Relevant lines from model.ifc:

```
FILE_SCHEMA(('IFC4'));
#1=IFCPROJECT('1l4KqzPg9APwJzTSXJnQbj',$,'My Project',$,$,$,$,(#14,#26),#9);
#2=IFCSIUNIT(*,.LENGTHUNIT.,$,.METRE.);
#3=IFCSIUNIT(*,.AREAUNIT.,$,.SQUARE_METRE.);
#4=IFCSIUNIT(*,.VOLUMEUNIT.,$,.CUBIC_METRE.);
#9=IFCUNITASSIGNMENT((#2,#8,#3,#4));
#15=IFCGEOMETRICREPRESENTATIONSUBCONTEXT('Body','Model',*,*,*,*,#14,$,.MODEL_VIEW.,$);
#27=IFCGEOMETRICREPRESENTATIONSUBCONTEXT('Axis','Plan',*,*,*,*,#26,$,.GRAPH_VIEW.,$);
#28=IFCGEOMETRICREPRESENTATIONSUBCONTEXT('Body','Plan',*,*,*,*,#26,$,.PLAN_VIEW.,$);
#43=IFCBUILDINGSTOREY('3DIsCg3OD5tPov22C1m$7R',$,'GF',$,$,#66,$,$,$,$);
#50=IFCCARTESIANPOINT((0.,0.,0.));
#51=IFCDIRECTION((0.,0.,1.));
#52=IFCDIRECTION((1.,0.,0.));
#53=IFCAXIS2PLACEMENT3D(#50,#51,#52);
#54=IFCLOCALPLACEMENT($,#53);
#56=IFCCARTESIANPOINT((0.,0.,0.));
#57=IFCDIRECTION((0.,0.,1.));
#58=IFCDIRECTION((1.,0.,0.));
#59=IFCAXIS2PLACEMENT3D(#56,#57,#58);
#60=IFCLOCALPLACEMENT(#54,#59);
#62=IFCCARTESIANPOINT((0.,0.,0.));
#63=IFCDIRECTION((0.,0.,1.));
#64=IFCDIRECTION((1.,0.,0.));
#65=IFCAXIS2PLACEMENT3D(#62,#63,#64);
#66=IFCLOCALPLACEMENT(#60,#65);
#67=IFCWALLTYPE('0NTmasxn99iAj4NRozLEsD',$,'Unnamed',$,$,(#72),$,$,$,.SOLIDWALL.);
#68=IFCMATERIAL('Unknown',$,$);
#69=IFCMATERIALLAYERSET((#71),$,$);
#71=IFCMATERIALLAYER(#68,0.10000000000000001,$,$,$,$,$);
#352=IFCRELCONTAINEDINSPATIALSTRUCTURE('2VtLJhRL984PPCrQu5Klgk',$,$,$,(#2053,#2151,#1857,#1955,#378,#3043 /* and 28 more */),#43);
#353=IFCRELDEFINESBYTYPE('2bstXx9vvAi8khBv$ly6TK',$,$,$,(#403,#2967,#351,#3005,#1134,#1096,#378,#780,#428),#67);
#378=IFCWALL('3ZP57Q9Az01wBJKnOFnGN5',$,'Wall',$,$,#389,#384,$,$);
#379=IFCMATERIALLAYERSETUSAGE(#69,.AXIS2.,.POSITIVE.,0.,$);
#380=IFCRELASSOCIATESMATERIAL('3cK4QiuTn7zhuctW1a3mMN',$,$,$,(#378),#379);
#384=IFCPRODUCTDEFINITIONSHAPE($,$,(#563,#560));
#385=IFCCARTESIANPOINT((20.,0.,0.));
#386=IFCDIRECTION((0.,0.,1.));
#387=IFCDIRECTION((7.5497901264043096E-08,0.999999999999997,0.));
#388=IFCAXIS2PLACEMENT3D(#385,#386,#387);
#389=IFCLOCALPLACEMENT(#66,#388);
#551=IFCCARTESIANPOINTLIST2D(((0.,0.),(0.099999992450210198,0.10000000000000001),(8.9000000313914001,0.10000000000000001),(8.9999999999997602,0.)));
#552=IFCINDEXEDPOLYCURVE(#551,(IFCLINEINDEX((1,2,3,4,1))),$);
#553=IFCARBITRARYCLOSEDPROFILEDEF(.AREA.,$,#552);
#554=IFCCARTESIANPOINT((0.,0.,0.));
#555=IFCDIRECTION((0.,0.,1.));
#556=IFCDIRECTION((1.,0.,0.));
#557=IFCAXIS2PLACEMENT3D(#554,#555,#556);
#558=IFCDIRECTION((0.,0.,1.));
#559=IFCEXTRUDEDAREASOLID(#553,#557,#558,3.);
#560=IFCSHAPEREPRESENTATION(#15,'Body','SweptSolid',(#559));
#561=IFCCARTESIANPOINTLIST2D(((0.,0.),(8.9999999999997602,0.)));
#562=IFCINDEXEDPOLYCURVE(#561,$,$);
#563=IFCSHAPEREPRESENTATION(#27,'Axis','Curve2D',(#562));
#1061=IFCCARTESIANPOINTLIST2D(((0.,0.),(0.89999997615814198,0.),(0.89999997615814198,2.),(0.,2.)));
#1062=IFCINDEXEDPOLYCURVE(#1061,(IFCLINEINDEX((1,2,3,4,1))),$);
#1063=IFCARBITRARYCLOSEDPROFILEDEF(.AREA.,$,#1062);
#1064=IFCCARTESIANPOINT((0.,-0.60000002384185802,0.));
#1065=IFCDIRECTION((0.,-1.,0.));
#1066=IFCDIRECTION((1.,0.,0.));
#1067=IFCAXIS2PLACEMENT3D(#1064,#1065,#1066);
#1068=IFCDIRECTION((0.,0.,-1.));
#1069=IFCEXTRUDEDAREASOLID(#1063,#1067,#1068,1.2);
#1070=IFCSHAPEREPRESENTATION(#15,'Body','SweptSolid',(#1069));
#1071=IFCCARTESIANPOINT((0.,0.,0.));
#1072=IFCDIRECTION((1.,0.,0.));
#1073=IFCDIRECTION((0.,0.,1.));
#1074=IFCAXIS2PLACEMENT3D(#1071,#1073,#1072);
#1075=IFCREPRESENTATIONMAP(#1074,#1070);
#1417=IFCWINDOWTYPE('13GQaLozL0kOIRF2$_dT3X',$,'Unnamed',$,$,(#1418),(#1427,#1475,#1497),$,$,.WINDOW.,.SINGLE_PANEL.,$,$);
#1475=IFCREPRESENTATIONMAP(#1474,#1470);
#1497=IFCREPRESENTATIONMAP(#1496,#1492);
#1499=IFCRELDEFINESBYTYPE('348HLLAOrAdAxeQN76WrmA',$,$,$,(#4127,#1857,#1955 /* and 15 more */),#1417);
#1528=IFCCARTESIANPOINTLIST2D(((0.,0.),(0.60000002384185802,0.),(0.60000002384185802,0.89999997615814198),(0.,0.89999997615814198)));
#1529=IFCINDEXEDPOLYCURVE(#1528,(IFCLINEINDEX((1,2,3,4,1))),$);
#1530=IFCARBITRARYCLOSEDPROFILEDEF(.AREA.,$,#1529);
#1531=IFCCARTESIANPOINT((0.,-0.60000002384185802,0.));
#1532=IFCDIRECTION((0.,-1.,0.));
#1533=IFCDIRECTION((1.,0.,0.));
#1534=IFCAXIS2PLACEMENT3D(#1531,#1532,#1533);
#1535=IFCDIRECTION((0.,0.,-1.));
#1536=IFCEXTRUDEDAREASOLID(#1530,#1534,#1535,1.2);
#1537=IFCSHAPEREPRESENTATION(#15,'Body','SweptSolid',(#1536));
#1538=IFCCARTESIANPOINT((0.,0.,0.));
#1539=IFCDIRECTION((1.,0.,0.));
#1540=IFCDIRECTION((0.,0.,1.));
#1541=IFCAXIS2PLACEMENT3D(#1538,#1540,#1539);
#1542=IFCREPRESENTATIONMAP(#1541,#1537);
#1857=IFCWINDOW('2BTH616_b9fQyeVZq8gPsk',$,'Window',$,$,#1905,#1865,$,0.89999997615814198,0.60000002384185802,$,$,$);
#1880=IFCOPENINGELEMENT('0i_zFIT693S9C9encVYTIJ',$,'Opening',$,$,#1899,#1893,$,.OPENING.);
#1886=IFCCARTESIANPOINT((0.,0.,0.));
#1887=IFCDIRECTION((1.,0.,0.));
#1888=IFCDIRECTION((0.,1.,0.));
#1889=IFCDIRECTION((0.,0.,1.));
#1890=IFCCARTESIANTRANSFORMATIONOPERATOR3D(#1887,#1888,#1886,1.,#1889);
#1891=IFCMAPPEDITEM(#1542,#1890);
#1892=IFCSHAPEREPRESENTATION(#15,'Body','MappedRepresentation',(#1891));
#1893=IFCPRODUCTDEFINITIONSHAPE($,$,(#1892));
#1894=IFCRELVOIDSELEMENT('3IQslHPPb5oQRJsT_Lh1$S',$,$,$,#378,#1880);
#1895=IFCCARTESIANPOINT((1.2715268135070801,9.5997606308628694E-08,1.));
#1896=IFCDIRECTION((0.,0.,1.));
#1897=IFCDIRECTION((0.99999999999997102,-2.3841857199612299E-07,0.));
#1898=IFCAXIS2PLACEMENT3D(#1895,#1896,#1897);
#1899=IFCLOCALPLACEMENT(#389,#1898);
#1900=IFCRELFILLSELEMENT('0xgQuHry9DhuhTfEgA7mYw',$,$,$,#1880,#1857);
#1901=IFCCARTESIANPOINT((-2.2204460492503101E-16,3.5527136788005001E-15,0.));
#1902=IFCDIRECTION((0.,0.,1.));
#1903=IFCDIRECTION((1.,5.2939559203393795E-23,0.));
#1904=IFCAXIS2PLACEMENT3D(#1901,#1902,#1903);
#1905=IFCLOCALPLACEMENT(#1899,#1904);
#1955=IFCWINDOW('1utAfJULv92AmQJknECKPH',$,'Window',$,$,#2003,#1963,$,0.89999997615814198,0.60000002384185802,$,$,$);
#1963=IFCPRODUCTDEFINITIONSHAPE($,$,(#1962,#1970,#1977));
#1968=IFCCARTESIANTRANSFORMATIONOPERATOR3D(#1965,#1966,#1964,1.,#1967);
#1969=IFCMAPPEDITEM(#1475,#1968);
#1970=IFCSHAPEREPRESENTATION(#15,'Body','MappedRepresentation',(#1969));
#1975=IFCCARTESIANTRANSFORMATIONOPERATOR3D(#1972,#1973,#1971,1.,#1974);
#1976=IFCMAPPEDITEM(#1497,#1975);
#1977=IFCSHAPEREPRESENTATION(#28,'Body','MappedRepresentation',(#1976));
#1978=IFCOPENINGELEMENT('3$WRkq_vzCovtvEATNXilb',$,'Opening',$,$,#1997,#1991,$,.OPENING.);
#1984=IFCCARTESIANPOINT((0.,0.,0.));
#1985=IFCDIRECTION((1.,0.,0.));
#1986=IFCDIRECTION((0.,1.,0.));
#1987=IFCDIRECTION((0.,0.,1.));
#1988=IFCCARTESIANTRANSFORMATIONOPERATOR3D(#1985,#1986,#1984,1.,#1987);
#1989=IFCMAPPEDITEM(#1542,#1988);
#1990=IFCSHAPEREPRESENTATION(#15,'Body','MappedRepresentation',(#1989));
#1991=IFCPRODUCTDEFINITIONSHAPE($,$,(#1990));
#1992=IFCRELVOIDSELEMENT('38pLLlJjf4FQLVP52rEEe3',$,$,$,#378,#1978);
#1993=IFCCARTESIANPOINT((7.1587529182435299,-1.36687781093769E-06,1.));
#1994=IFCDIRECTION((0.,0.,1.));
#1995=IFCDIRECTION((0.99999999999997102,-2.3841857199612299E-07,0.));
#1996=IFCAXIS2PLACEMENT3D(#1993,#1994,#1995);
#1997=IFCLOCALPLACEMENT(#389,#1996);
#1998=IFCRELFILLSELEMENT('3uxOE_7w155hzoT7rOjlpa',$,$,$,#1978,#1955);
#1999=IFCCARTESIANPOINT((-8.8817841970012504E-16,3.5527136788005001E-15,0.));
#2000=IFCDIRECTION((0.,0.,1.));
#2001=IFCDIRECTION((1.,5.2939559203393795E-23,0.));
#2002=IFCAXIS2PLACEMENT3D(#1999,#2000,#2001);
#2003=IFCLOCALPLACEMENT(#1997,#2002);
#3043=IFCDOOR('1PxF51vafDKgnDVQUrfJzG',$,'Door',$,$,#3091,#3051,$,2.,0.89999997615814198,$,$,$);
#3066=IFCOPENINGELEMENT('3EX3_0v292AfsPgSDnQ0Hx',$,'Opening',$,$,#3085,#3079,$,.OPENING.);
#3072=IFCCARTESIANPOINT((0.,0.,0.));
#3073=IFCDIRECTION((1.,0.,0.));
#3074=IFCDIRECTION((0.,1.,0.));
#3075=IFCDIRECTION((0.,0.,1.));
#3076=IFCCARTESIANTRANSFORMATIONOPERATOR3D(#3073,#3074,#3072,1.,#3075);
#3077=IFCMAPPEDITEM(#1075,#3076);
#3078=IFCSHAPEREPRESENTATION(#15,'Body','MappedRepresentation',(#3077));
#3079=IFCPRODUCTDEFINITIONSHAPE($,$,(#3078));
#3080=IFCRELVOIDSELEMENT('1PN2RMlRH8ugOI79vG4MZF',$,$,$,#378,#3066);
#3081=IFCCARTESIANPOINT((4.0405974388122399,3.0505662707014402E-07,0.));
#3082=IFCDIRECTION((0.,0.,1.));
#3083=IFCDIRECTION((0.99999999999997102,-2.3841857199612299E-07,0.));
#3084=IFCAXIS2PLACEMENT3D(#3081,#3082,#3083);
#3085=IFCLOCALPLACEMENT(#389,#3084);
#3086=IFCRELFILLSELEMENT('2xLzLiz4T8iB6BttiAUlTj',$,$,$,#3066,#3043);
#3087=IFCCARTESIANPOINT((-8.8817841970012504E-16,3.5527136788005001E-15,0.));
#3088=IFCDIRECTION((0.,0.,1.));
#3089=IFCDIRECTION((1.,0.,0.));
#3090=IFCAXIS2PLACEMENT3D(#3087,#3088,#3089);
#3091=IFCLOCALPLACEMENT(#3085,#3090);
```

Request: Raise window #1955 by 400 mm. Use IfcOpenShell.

```python
import numpy as np
import ifcopenshell
import ifcopenshell.api.geometry
import ifcopenshell.util.placement
import ifcopenshell.util.unit

model = ifcopenshell.open("model.ifc")
unit_scale = ifcopenshell.util.unit.calculate_unit_scale(model)

window = model.by_id(1955)
opening = window.FillsVoids[0].RelatingOpeningElement
dz = 0.4

shift = np.array([0.0, 0.0, dz])
# The window is placed relative to its opening, so it follows when the opening moves.
matrix = ifcopenshell.util.placement.get_local_placement(opening.ObjectPlacement)
matrix[:3, 3] += shift
ifcopenshell.api.geometry.edit_object_placement(
    model, product=opening, matrix=matrix, is_si=False, should_transform_children=True
)

print(f"moved by {dz * unit_scale:+.3f} m")

model.write("model_updated.ifc")
```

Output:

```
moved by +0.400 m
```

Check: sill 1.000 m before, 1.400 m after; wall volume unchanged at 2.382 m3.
